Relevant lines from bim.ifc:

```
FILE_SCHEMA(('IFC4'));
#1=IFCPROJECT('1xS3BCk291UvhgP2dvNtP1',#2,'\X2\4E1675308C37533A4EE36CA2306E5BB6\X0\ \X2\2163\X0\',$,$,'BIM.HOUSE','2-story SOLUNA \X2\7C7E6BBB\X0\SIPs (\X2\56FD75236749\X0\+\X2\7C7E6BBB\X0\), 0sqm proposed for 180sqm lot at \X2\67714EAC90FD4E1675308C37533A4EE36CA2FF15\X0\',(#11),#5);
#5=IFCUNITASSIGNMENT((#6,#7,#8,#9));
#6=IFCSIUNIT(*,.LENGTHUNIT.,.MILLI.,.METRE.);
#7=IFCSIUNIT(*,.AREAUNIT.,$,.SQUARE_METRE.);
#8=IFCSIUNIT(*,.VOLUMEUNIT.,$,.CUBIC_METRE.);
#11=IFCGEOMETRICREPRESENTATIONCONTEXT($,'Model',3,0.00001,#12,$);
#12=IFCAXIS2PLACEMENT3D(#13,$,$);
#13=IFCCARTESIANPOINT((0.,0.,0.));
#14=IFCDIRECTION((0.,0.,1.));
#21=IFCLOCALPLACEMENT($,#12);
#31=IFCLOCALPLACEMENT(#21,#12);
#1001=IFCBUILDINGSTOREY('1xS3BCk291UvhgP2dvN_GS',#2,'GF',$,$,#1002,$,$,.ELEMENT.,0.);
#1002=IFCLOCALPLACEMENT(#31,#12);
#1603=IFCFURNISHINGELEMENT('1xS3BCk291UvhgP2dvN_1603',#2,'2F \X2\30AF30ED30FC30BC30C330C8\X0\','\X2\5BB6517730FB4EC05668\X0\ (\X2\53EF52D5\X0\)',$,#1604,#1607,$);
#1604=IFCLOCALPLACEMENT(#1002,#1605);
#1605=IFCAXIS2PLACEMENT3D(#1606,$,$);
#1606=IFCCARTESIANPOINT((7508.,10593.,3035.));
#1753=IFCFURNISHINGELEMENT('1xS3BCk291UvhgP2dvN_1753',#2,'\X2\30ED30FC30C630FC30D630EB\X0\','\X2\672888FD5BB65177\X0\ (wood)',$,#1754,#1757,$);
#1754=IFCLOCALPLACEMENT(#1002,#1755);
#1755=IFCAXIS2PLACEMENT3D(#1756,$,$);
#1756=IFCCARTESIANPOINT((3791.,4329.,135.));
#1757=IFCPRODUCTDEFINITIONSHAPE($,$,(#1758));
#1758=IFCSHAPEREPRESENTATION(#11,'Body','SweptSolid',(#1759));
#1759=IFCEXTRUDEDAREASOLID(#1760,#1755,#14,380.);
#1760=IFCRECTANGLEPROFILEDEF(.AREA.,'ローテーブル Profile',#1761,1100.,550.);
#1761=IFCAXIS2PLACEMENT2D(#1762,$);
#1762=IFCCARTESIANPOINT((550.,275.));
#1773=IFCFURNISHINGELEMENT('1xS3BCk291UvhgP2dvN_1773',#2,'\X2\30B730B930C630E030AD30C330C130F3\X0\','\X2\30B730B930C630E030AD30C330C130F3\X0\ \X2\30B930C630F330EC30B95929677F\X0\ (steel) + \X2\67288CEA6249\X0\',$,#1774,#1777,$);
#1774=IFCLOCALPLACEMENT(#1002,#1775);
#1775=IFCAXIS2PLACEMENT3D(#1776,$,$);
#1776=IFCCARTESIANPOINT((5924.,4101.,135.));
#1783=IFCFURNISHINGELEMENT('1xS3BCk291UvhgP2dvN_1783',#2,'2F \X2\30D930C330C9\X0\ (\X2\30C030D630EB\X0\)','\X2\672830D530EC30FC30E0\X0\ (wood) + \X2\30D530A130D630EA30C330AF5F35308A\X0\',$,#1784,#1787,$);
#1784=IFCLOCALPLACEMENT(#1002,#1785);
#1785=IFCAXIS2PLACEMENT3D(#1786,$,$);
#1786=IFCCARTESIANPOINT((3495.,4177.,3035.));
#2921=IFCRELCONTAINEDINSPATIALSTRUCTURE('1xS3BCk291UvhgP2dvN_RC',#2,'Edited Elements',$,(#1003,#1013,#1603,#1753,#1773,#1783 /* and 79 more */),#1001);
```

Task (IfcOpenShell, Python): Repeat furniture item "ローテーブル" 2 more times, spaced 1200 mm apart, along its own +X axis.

```python
import ifcopenshell
import ifcopenshell.api.geometry
import ifcopenshell.api.root
import ifcopenshell.util.element
import ifcopenshell.util.placement
import ifcopenshell.util.unit

model = ifcopenshell.open("bim.ifc")
unit_scale = ifcopenshell.util.unit.calculate_unit_scale(model)


def reuse_history(source, copy):
    """copy_class also copies each property set's owner history, people and application; keep the originals."""
    for rel in copy.IsDefinedBy:
        if rel.is_a("IfcRelDefinesByProperties") and (history := rel.RelatingPropertyDefinition.OwnerHistory):
            rel.RelatingPropertyDefinition.OwnerHistory = source.OwnerHistory
            ifcopenshell.util.element.remove_deep2(model, history)


source = model.by_guid("1xS3BCk291UvhgP2dvN_1753")
base = ifcopenshell.util.placement.get_local_placement(source.ObjectPlacement)
step = base[:3, 0] * 1.2 / unit_scale

for i in range(1, 3):
    copy = ifcopenshell.api.root.copy_class(model, product=source)
    copy.Representation = ifcopenshell.util.element.copy_deep(
        model, source.Representation, exclude=["IfcGeometricRepresentationContext", "IfcRepresentationMap"]
    )
    reuse_history(source, copy)
    matrix = base.copy()
    matrix[:3, 3] += i * step
    print("added at", matrix[:3, 3].round(3) + 0.0)
    ifcopenshell.api.geometry.edit_object_placement(model, product=copy, matrix=matrix, is_si=False)

model.write("bim_v2.ifc")
```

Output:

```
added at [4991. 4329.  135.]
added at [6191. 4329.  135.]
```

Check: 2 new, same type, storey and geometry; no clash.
